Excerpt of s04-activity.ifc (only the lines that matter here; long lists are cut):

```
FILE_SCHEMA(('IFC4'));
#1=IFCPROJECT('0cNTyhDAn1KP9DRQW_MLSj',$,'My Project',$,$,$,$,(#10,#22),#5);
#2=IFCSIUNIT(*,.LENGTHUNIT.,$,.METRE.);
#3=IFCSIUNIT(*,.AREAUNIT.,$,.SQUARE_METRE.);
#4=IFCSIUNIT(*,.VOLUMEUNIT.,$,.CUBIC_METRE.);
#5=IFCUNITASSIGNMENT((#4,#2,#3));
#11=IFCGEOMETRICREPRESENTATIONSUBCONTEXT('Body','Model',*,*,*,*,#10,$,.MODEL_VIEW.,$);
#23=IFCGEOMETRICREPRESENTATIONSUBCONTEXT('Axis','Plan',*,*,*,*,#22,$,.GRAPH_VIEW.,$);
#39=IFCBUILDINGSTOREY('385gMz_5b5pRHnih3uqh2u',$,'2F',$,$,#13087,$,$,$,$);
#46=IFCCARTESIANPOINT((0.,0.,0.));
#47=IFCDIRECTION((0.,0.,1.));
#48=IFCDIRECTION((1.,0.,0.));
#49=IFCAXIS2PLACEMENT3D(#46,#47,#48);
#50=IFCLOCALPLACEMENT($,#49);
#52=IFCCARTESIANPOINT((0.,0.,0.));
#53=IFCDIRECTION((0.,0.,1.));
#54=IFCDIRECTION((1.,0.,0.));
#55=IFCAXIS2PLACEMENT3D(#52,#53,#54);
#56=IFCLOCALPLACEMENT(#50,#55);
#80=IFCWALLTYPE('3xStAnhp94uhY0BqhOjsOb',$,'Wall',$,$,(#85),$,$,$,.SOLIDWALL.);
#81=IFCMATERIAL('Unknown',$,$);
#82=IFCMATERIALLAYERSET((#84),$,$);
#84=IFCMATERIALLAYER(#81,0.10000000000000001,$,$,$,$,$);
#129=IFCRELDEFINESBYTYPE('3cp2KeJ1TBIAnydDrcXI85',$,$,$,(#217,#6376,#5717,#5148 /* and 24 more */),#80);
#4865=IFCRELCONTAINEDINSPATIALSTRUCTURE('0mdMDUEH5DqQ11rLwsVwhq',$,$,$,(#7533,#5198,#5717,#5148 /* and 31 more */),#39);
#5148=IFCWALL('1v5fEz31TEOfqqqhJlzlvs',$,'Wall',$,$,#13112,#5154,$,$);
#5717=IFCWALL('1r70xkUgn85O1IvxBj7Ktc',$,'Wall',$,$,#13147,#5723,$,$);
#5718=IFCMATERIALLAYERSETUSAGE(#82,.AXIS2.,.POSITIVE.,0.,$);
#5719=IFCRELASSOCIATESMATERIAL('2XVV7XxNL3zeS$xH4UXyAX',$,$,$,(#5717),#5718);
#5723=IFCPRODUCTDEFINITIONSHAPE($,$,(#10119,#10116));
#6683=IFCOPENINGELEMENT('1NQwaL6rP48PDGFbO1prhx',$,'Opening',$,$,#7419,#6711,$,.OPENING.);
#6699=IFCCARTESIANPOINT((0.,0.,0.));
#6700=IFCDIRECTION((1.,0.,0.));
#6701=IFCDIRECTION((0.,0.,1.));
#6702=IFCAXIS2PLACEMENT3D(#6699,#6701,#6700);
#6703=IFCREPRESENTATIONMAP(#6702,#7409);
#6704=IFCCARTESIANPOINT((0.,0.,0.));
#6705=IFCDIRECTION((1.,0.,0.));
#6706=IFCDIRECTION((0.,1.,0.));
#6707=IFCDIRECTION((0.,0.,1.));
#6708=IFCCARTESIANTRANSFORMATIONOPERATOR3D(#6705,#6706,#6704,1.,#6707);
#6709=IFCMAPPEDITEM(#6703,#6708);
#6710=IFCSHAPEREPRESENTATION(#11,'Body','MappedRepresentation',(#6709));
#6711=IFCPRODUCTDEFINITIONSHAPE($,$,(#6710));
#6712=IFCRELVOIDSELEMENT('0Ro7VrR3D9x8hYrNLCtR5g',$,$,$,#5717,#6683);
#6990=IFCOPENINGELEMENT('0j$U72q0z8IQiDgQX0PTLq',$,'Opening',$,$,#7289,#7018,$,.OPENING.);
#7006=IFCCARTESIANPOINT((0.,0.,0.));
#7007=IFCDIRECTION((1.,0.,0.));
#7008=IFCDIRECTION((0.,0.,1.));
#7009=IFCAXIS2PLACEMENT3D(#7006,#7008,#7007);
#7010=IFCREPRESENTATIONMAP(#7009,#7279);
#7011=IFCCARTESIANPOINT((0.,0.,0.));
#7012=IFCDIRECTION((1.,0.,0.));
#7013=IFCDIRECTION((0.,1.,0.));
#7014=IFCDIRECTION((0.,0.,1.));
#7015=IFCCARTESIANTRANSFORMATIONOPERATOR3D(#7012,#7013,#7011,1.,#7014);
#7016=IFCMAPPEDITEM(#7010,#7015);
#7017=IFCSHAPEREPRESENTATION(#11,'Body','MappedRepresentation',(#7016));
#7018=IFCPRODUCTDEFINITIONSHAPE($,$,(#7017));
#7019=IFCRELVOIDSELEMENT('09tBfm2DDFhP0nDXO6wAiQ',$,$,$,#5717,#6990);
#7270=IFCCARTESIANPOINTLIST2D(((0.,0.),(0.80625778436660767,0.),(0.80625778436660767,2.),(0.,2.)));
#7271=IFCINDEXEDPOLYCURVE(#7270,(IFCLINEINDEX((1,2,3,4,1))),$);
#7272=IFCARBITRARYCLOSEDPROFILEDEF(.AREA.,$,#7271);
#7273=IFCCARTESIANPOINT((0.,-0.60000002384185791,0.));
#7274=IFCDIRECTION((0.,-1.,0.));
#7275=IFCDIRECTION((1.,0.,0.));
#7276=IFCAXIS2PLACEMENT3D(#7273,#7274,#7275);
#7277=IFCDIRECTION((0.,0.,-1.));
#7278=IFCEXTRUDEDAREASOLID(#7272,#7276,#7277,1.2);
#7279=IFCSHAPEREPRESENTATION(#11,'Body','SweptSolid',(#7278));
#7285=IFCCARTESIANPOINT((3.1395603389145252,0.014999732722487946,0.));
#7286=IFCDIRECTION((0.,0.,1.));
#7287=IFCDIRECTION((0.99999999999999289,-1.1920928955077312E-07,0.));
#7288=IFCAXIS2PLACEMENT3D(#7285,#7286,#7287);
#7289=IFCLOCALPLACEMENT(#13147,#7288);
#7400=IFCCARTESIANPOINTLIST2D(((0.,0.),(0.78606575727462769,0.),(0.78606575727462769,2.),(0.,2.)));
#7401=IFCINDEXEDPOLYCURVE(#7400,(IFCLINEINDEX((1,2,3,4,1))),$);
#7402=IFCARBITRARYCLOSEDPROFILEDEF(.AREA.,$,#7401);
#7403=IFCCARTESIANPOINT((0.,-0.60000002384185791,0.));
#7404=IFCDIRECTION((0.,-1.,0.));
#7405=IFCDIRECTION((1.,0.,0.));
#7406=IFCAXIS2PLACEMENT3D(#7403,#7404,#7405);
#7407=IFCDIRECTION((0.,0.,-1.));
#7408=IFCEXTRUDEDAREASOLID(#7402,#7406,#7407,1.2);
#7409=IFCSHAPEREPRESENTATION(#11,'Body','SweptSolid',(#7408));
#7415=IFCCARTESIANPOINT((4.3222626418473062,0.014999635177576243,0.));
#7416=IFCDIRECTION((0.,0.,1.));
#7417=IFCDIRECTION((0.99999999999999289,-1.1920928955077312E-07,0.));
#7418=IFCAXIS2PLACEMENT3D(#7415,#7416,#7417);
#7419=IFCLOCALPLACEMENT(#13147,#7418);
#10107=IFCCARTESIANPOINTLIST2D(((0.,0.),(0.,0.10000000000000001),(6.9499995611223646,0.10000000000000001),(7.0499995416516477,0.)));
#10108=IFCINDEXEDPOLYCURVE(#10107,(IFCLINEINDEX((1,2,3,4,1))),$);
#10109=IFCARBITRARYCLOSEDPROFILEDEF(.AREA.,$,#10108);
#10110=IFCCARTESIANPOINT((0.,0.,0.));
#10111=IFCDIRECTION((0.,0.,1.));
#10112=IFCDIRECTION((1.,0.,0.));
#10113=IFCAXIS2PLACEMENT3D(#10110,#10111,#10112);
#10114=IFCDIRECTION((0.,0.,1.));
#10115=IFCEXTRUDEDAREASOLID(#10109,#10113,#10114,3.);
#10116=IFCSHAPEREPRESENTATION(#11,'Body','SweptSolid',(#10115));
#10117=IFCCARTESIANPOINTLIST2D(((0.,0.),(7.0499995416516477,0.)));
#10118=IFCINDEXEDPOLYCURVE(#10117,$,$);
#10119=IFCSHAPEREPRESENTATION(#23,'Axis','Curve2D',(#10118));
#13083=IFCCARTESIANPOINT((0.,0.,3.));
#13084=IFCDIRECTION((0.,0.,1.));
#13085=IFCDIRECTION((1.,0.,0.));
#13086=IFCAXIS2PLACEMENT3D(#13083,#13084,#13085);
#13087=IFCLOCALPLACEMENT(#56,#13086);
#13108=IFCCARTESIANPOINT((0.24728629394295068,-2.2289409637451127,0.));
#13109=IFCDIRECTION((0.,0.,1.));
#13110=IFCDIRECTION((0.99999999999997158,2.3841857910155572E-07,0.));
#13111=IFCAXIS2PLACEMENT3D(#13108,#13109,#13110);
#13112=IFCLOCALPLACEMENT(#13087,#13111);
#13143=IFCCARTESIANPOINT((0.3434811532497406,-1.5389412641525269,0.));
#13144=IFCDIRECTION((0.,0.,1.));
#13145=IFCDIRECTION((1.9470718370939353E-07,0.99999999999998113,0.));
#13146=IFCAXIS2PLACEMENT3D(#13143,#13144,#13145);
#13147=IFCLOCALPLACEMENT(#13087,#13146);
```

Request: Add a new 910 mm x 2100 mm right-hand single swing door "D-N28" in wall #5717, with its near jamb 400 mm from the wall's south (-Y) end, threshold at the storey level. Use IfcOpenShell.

```python
import numpy as np
import ifcopenshell
import ifcopenshell.api.feature
import ifcopenshell.api.geometry
import ifcopenshell.api.root
import ifcopenshell.api.spatial
import ifcopenshell.geom
import ifcopenshell.util.element
import ifcopenshell.util.placement
import ifcopenshell.util.representation
import ifcopenshell.util.shape
import ifcopenshell.util.unit

model = ifcopenshell.open("s04-activity.ifc")
unit_scale = ifcopenshell.util.unit.calculate_unit_scale(model)
settings = ifcopenshell.geom.settings()


def volume(element):
    """Net volume in cubic metres, openings subtracted."""
    shape = ifcopenshell.geom.create_shape(settings, element)
    return ifcopenshell.util.shape.get_volume(shape.geometry)


wall = model.by_guid("1r70xkUgn85O1IvxBj7Ktc")
storey = ifcopenshell.util.element.get_container(wall, ifc_class="IfcBuildingStorey")
context = ifcopenshell.util.representation.get_context(model, "Model", "Body", "MODEL_VIEW")
before = volume(wall)

width, height, from_end, sill = 0.91, 2.1, 0.4, 0.0  # metres

# The wall runs along its own X axis, and the end named is its -X end.
wall_shape = ifcopenshell.geom.create_shape(settings, wall)
x, y, z = ifcopenshell.util.shape.get_vertices(wall_shape.geometry).T
start = x.min() + from_end
face, thickness = float(y.min()), float(y.max() - y.min())
wall_matrix = ifcopenshell.util.placement.get_local_placement(wall.ObjectPlacement)
level = ifcopenshell.util.placement.get_local_placement(storey.ObjectPlacement)[2, 3]


def in_wall(x, y):
    """Placement at x, y metres in the wall's axes, at sill height."""
    matrix = wall_matrix.copy()
    matrix[:, 3] = wall_matrix @ np.array([x / unit_scale, y / unit_scale, 0.0, 1.0])
    matrix[2, 3] = level + sill / unit_scale
    return matrix


# Opening: a box that overshoots both wall faces by 50 mm.
opening = ifcopenshell.api.root.create_entity(model, ifc_class="IfcOpeningElement", predefined_type="OPENING")
box = ifcopenshell.api.geometry.add_wall_representation(
    model, context=context, length=width, height=height, thickness=thickness + 0.1
)
ifcopenshell.api.geometry.assign_representation(model, product=opening, representation=box)
ifcopenshell.api.geometry.edit_object_placement(model, product=opening, matrix=in_wall(start, face - 0.05), is_si=False)
ifcopenshell.api.feature.add_feature(model, feature=opening, element=wall)

door = ifcopenshell.api.root.create_entity(model, ifc_class="IfcDoor", name="D-N28", predefined_type="DOOR")
door.OverallWidth, door.OverallHeight = width / unit_scale, height / unit_scale
door.OperationType = "SINGLE_SWING_RIGHT"
body = ifcopenshell.api.geometry.add_door_representation(
    model,
    context=context,
    overall_width=door.OverallWidth,
    overall_height=door.OverallHeight,
    operation_type="SINGLE_SWING_RIGHT",
    lining_properties={"LiningDepth": thickness / unit_scale, "ThresholdDepth": thickness / unit_scale},
)
ifcopenshell.api.geometry.assign_representation(model, product=door, representation=body)
ifcopenshell.api.spatial.assign_container(model, products=[door], relating_structure=storey)
ifcopenshell.api.feature.add_filling(model, opening=opening, element=door)

# The lining spans the wall, so the door starts at the wall face.
ifcopenshell.api.geometry.edit_object_placement(model, product=door, matrix=in_wall(start, face), is_si=False)

after = volume(wall)

print(f"wall volume {before:.3f} -> {after:.3f} m3")

model.write("s04-activity_v2.ifc")
```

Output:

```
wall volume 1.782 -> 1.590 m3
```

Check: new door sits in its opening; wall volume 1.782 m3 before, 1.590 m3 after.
